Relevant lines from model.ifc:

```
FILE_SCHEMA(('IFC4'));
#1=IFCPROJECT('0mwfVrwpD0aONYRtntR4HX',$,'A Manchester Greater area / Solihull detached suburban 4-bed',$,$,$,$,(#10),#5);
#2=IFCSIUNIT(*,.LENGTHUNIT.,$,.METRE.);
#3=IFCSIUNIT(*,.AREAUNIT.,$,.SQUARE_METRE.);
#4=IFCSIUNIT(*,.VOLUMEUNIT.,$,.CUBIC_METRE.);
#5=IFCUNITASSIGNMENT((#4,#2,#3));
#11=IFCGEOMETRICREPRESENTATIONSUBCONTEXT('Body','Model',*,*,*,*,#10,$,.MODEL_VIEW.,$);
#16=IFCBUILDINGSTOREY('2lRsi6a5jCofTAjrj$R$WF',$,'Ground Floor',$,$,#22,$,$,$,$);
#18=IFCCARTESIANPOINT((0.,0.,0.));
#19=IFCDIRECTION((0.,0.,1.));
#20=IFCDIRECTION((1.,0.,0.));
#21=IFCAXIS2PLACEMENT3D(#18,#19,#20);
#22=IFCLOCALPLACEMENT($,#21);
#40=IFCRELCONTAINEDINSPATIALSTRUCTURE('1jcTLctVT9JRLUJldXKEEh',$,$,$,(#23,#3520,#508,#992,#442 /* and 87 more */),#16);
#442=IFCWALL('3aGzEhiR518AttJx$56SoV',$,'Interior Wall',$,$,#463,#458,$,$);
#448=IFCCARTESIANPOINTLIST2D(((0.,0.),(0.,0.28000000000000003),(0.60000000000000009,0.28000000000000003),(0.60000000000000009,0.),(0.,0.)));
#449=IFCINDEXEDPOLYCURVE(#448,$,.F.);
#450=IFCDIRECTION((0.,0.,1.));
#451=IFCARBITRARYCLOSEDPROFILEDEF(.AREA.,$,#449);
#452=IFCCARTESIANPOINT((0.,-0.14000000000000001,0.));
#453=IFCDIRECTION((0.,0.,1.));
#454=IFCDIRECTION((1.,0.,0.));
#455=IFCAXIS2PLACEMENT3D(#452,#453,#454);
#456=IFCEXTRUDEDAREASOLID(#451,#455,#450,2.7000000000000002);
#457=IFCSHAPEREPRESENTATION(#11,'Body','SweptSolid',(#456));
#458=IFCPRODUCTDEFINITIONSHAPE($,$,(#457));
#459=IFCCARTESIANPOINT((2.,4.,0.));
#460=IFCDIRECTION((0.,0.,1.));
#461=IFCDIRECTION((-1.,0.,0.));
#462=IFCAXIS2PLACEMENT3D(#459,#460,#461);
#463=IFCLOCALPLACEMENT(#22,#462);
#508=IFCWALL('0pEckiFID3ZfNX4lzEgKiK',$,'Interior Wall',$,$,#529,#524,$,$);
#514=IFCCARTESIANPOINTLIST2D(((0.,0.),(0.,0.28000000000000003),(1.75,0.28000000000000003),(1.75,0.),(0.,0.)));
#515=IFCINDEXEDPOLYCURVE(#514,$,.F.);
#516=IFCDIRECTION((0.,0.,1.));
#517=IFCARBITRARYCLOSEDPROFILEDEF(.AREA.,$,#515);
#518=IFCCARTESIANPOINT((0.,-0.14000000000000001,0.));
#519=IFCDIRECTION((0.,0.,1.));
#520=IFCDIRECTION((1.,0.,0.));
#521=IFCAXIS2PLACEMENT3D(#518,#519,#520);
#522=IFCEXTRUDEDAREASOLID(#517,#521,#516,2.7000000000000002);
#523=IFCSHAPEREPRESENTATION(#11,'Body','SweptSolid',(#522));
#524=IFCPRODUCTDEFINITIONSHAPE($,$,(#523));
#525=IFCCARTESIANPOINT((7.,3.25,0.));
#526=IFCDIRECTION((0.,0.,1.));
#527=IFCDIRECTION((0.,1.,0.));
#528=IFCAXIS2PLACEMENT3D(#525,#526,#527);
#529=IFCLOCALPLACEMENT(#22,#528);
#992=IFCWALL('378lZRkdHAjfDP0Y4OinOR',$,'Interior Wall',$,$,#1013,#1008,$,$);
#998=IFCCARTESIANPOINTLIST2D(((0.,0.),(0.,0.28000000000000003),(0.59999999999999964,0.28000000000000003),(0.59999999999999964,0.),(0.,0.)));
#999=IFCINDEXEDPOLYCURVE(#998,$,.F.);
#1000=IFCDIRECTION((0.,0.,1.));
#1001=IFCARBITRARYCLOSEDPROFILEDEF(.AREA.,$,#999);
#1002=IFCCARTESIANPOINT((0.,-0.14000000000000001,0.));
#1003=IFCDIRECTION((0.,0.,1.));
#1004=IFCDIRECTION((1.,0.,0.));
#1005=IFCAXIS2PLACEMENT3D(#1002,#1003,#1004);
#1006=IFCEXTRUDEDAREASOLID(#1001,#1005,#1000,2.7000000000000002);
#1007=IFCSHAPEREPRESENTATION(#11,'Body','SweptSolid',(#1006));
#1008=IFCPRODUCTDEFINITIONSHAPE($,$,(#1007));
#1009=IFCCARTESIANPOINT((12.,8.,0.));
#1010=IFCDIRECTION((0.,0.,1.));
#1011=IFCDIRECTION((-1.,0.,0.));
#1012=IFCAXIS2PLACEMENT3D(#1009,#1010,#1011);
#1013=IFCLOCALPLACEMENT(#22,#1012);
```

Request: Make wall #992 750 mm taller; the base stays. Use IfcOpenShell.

```python
import ifcopenshell
import ifcopenshell.geom
import ifcopenshell.util.representation
import ifcopenshell.util.shape
import ifcopenshell.util.unit

model = ifcopenshell.open("model.ifc")
unit_scale = ifcopenshell.util.unit.calculate_unit_scale(model)
settings = ifcopenshell.geom.settings()


def volume(element):
    """Net volume in cubic metres, openings subtracted."""
    shape = ifcopenshell.geom.create_shape(settings, element)
    return ifcopenshell.util.shape.get_volume(shape.geometry)


wall = model.by_guid("378lZRkdHAjfDP0Y4OinOR")
before = volume(wall)

body = ifcopenshell.util.representation.get_representation(wall, "Model", "Body")
solid = body.Items[0]
old_height = solid.Depth
solid.Depth += 0.75 / unit_scale
after = volume(wall)

print(f"height {old_height:g} -> {solid.Depth:g}, volume {before:.3f} -> {after:.3f} m3")

model.write("model_rev.ifc")
```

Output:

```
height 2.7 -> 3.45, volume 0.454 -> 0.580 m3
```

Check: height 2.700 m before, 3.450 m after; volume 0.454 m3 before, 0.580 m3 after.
